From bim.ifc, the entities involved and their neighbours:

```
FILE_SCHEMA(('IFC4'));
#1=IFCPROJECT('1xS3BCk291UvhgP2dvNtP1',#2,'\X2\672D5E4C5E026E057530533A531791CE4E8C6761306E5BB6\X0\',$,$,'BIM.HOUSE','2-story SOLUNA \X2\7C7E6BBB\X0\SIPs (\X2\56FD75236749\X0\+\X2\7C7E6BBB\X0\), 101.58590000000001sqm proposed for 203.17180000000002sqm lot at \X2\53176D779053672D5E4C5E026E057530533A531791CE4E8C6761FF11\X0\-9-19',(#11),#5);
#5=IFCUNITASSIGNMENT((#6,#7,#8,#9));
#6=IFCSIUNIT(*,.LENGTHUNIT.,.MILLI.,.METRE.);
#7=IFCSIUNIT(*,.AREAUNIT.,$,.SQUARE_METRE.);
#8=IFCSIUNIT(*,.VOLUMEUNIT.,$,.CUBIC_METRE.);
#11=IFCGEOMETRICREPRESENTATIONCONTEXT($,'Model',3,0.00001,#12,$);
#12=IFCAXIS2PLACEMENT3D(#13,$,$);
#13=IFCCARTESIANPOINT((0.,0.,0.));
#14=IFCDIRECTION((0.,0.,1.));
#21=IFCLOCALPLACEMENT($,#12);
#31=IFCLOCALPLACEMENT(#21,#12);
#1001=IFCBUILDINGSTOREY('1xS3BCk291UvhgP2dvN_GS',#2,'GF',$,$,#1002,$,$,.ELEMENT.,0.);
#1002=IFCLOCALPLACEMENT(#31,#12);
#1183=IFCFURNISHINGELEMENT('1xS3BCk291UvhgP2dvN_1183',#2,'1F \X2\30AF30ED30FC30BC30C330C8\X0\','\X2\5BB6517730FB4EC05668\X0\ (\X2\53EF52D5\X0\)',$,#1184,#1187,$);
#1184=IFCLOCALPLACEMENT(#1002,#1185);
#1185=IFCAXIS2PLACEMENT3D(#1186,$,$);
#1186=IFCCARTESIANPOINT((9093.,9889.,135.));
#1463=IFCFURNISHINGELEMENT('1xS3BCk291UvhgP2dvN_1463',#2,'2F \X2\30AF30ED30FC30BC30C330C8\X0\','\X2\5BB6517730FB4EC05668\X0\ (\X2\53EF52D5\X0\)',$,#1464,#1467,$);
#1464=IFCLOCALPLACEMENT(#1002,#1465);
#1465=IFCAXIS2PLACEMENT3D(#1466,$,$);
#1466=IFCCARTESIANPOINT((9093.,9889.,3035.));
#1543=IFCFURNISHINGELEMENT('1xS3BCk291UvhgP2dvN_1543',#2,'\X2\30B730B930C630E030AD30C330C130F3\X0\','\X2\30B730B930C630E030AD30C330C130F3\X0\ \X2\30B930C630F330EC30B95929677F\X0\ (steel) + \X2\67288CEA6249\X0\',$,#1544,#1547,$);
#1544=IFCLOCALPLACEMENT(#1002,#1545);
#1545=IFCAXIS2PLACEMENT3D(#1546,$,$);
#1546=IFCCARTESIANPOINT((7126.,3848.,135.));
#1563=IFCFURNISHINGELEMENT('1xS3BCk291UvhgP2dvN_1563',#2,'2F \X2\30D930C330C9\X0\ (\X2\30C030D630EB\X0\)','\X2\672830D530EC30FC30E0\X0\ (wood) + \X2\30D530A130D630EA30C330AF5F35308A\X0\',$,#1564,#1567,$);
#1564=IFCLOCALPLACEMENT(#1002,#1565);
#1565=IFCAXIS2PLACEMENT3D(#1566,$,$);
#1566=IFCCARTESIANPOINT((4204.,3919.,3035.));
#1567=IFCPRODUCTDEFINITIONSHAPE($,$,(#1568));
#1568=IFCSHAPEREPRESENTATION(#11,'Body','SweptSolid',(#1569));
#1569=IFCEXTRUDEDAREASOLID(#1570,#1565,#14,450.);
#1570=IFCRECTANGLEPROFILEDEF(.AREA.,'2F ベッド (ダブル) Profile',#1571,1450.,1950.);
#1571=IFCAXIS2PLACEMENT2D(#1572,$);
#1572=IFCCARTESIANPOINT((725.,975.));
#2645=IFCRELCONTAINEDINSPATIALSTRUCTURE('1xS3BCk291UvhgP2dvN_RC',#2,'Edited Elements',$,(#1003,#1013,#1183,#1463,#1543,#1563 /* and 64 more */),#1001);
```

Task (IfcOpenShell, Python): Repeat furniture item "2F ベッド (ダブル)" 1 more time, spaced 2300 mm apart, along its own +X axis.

```python
import ifcopenshell
import ifcopenshell.api.geometry
import ifcopenshell.api.root
import ifcopenshell.util.element
import ifcopenshell.util.placement
import ifcopenshell.util.unit

model = ifcopenshell.open("bim.ifc")
unit_scale = ifcopenshell.util.unit.calculate_unit_scale(model)


def reuse_history(source, copy):
    """copy_class also copies each property set's owner history, people and application; keep the originals."""
    for rel in copy.IsDefinedBy:
        if rel.is_a("IfcRelDefinesByProperties") and (history := rel.RelatingPropertyDefinition.OwnerHistory):
            rel.RelatingPropertyDefinition.OwnerHistory = source.OwnerHistory
            ifcopenshell.util.element.remove_deep2(model, history)


source = model.by_guid("1xS3BCk291UvhgP2dvN_1563")
base = ifcopenshell.util.placement.get_local_placement(source.ObjectPlacement)
step = base[:3, 0] * 2.3 / unit_scale

for i in range(1, 2):
    copy = ifcopenshell.api.root.copy_class(model, product=source)
    copy.Representation = ifcopenshell.util.element.copy_deep(
        model, source.Representation, exclude=["IfcGeometricRepresentationContext", "IfcRepresentationMap"]
    )
    reuse_history(source, copy)
    matrix = base.copy()
    matrix[:3, 3] += i * step
    print("added at", matrix[:3, 3].round(3) + 0.0)
    ifcopenshell.api.geometry.edit_object_placement(model, product=copy, matrix=matrix, is_si=False)

model.write("bim_rev.ifc")
```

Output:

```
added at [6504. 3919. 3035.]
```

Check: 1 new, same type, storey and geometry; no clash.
